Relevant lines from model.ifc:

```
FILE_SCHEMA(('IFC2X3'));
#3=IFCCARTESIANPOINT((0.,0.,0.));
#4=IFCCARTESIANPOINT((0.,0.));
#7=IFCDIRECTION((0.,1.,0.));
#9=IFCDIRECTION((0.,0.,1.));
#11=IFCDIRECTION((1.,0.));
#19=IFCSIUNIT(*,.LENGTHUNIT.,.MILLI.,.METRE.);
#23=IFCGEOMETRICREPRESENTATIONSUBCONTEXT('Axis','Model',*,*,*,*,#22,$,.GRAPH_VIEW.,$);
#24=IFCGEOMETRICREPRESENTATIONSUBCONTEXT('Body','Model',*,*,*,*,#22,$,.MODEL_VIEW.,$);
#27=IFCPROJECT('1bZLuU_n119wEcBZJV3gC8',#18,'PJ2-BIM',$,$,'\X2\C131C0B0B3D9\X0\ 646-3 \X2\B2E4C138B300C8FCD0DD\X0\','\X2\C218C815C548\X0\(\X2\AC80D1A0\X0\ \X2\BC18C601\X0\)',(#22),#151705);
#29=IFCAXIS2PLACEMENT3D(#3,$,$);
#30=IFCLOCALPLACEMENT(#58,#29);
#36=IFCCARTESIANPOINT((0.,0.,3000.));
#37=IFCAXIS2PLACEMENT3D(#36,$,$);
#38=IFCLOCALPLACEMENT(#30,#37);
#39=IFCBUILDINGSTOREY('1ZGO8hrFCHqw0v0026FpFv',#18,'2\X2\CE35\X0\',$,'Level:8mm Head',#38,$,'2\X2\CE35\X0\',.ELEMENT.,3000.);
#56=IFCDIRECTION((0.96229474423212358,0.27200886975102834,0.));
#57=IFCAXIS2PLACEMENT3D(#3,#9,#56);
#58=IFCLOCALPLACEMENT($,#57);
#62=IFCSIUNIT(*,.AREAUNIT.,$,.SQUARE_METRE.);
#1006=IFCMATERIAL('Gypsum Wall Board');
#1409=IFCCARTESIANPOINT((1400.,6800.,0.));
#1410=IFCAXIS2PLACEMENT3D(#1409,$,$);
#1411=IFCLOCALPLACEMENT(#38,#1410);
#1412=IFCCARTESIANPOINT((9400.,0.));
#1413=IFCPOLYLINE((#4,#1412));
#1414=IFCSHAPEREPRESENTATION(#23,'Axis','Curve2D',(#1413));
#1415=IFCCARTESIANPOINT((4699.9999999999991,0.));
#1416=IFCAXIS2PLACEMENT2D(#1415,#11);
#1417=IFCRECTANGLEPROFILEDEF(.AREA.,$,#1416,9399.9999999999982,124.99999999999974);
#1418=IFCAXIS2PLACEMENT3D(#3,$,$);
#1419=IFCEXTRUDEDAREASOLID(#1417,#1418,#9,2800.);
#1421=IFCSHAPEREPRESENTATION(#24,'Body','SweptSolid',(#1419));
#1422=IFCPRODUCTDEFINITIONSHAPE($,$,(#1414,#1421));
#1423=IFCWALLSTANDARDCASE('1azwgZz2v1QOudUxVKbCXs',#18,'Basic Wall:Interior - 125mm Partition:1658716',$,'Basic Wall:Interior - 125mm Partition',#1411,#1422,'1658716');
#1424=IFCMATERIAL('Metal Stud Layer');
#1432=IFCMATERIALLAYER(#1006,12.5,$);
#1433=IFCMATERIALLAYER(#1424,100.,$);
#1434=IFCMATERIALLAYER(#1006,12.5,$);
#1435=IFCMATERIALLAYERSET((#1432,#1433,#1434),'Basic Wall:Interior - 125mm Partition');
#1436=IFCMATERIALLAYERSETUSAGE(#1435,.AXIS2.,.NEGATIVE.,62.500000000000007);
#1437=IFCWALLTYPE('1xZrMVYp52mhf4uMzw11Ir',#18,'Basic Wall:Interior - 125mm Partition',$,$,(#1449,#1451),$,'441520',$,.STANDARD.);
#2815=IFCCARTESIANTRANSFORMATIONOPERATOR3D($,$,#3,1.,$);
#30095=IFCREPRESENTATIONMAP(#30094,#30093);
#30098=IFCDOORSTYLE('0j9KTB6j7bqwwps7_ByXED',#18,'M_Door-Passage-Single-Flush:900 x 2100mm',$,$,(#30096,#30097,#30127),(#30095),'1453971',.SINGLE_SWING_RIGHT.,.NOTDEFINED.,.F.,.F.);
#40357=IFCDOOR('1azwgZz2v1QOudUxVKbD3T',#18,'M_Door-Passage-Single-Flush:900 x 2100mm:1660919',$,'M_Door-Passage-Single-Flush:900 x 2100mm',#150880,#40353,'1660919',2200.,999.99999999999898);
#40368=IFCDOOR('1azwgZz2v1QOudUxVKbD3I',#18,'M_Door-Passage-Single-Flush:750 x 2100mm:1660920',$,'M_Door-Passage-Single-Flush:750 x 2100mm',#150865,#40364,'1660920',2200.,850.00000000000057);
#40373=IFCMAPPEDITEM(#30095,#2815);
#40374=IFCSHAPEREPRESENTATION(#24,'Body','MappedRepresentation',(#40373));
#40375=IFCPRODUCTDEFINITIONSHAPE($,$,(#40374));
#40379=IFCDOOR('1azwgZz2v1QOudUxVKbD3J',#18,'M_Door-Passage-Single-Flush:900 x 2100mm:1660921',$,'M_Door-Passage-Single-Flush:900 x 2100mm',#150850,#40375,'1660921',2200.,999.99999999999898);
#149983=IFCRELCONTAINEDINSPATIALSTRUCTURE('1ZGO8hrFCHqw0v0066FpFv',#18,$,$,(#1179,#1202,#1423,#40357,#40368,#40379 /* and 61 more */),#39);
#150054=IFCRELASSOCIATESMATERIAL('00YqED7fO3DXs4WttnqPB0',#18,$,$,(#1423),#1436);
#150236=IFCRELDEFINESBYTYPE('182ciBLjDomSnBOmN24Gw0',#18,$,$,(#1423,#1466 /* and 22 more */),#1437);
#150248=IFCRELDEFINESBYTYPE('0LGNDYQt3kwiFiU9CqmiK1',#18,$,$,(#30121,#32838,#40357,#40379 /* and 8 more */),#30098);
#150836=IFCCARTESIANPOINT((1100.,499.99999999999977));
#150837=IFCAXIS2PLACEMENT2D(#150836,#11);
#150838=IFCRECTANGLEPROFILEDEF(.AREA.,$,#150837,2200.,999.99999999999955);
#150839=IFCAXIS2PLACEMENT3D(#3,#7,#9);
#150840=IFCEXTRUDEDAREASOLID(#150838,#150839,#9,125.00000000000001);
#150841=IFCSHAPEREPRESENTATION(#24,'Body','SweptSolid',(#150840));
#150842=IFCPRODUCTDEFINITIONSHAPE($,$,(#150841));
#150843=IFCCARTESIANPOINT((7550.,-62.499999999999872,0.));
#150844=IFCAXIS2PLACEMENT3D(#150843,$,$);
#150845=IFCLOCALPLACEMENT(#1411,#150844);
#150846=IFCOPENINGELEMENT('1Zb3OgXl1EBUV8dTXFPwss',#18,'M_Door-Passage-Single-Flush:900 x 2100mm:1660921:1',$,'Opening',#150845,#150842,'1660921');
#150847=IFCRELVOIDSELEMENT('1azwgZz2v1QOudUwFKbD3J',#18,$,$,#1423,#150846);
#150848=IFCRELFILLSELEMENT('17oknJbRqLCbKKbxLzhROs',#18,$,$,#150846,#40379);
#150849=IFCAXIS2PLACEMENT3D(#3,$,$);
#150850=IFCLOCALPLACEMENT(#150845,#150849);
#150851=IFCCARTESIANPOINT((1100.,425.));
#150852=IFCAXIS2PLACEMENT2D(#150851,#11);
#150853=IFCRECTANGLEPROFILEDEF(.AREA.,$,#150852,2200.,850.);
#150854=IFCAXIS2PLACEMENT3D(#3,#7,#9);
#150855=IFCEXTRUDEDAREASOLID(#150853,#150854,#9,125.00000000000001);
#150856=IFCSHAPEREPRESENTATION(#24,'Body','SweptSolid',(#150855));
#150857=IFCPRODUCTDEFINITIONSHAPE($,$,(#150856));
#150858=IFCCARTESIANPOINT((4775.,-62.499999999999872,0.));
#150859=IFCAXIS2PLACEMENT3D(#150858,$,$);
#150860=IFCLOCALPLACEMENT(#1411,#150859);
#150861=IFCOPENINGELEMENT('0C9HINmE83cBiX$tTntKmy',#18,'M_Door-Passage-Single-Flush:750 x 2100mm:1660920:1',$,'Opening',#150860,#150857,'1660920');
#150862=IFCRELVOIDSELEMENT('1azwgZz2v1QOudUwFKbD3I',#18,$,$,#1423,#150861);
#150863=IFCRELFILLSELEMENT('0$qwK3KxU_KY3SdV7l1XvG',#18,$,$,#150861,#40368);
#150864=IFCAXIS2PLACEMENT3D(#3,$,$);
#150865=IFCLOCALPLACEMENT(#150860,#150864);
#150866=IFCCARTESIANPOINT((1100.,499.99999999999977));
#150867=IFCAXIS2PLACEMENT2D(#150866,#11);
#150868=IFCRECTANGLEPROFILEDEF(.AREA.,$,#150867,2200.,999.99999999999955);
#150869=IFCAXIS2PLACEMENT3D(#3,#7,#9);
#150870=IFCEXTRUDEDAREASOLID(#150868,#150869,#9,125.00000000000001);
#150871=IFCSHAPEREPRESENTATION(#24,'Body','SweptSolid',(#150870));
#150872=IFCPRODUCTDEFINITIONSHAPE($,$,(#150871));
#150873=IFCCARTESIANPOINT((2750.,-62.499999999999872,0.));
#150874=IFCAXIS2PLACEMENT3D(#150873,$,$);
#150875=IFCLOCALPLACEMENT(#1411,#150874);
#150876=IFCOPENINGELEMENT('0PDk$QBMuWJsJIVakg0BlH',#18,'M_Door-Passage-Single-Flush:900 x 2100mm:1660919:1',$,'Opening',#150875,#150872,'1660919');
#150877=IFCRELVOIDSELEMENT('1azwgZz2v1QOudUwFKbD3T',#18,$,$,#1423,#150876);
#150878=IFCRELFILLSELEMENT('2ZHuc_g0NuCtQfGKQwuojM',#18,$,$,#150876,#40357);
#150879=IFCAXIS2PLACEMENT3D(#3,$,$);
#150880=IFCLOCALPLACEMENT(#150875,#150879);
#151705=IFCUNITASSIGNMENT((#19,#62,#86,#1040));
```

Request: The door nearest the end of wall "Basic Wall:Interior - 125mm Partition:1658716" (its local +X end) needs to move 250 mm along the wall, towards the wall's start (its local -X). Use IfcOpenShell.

```python
import ifcopenshell
import ifcopenshell.api.geometry
import ifcopenshell.util.placement
import ifcopenshell.util.unit

model = ifcopenshell.open("model.ifc")
unit_scale = ifcopenshell.util.unit.calculate_unit_scale(model)

door = model.by_guid("1azwgZz2v1QOudUxVKbD3J")
opening = door.FillsVoids[0].RelatingOpeningElement
wall = opening.VoidsElements[0].RelatingBuildingElement

wall_matrix = ifcopenshell.util.placement.get_local_placement(wall.ObjectPlacement)
shift = wall_matrix[:3, 0] * -0.25 / unit_scale
before = ifcopenshell.util.placement.get_local_placement(door.ObjectPlacement)[:3, 3].copy()

# The door is placed relative to its opening, so it follows when the opening moves.
matrix = ifcopenshell.util.placement.get_local_placement(opening.ObjectPlacement)
matrix[:3, 3] += shift
ifcopenshell.api.geometry.edit_object_placement(
    model, product=opening, matrix=matrix, is_si=False, should_transform_children=True
)

after = ifcopenshell.util.placement.get_local_placement(door.ObjectPlacement)[:3, 3]
print("door moved by", (after - before).round(3) + 0.0)

model.write("model-out.ifc")
```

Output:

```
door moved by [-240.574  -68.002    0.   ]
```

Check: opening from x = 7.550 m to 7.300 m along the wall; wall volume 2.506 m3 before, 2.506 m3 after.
